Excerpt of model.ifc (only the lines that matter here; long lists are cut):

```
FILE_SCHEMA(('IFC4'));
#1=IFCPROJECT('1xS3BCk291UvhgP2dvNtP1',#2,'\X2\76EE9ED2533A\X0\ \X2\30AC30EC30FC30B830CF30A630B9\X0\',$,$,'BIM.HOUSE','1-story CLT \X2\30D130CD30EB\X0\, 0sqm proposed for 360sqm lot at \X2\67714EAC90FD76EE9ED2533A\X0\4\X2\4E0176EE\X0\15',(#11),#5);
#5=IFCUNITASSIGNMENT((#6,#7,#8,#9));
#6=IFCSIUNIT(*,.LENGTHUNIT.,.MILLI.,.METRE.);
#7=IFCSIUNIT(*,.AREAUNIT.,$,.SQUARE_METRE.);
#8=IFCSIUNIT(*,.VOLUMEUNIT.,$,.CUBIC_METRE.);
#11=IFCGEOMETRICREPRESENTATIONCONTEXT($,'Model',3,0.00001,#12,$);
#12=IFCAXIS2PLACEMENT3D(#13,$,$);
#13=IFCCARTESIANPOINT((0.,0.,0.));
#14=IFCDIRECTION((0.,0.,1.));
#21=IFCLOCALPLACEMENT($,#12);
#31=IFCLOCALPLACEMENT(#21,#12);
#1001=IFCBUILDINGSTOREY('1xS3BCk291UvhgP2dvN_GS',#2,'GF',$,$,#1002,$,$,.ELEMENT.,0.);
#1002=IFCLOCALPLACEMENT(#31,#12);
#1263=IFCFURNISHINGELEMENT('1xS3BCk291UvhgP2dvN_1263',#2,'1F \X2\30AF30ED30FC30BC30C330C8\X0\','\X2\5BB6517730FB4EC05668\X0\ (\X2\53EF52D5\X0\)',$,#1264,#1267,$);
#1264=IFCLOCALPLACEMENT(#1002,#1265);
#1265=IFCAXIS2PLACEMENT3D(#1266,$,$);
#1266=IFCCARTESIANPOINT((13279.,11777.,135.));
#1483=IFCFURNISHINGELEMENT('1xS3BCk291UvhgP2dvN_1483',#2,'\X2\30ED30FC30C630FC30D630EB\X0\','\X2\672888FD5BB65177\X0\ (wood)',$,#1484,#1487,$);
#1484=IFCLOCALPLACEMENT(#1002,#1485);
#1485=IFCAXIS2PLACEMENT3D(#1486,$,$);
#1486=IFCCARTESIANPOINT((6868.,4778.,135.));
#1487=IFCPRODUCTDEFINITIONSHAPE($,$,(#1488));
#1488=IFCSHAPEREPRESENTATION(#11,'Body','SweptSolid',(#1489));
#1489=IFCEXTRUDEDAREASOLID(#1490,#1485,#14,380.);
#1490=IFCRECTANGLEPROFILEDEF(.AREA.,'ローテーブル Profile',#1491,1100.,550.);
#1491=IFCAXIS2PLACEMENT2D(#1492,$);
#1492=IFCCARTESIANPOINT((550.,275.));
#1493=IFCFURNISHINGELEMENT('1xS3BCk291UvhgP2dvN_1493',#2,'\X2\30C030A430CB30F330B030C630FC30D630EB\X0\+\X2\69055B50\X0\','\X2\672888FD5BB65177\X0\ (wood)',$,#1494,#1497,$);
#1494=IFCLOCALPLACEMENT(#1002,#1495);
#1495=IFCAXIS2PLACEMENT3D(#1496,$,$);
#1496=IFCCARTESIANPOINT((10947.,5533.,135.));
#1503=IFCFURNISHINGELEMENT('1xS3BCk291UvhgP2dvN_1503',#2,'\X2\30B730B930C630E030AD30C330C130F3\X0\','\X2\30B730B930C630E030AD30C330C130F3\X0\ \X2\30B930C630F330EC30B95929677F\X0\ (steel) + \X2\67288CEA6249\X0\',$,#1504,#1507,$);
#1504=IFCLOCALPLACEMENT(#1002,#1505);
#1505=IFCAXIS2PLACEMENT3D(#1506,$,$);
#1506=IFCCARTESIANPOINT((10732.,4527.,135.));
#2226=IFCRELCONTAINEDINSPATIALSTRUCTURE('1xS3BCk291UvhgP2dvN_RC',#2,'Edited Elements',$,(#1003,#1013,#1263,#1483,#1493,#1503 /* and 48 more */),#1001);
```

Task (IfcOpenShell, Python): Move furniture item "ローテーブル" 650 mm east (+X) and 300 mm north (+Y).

```python
import ifcopenshell
import ifcopenshell.api.geometry
import ifcopenshell.util.placement
import ifcopenshell.util.unit

model = ifcopenshell.open("model.ifc")
unit_scale = ifcopenshell.util.unit.calculate_unit_scale(model)

item = model.by_guid("1xS3BCk291UvhgP2dvN_1483")
matrix = ifcopenshell.util.placement.get_local_placement(item.ObjectPlacement)
matrix[0, 3] += 0.65 / unit_scale
matrix[1, 3] += 0.3 / unit_scale
ifcopenshell.api.geometry.edit_object_placement(model, product=item, matrix=matrix, is_si=False)

print(ifcopenshell.util.placement.get_local_placement(item.ObjectPlacement).round(3) + 0.0)

model.write("model_updated.ifc")
```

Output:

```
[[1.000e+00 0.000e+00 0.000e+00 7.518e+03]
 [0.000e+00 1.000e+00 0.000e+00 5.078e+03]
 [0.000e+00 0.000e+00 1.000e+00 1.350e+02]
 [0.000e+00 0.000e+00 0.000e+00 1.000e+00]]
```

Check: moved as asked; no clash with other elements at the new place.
